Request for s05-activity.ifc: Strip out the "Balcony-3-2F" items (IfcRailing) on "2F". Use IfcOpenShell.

First a look at what the model holds.

```python
import ifcopenshell
import ifcopenshell.util.element

model = ifcopenshell.open("s05-activity.ifc")
print(model.schema)
storey = next(s for s in model.by_type("IfcBuildingStorey") if s.Name == "2F")
railings = [e for e in ifcopenshell.util.element.get_decomposition(storey) if e.is_a("IfcRailing")]
seen = {}
for e in railings:
    element_type = ifcopenshell.util.element.get_type(e)
    name = element_type.Name if element_type not in (None, e) else None
    seen[name] = seen.get(name, 0) + 1
for name, count in sorted(seen.items(), key=str):
    print(count, "x", name)
```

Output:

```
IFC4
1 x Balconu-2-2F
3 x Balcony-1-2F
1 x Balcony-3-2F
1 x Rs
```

```python
import ifcopenshell
import ifcopenshell.api.root
import ifcopenshell.util.element

model = ifcopenshell.open("s05-activity.ifc")

storey = next(s for s in model.by_type("IfcBuildingStorey") if s.Name == "2F")
railings = [e for e in ifcopenshell.util.element.get_decomposition(storey) if e.is_a("IfcRailing")]
targets = [e for e in railings if (t := ifcopenshell.util.element.get_type(e)) not in (None, e) and t.Name == "Balcony-3-2F"]

for e in targets:
    ifcopenshell.api.root.remove_product(model, product=e)
print(len(targets), "removed")

model.write("s05-activity_v2.ifc")
```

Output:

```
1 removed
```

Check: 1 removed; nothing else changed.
